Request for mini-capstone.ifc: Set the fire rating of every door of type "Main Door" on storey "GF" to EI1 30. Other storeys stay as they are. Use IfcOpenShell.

First a look at what the model holds.

```python
import ifcopenshell
import ifcopenshell.util.element

model = ifcopenshell.open("mini-capstone.ifc")
print(model.schema)
storey = next(s for s in model.by_type("IfcBuildingStorey") if s.Name == "GF")
doors = [e for e in ifcopenshell.util.element.get_decomposition(storey) if e.is_a("IfcDoor")]
seen = {}
for e in doors:
    element_type = ifcopenshell.util.element.get_type(e)
    key = (element_type.Name if element_type != e and element_type else None, ifcopenshell.util.element.get_pset(e, "Pset_DoorCommon", "FireRating"))
    seen[key] = seen.get(key, 0) + 1
for (name, value), count in sorted(seen.items(), key=str):
    print(count, "x", name, "|", value)
```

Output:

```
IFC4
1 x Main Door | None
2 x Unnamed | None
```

```python
import ifcopenshell
import ifcopenshell.api.pset
import ifcopenshell.util.element

model = ifcopenshell.open("mini-capstone.ifc")

storey = next(s for s in model.by_type("IfcBuildingStorey") if s.Name == "GF")
doors = [e for e in ifcopenshell.util.element.get_decomposition(storey) if e.is_a("IfcDoor")]

count = 0
for e in doors:
    element_type = ifcopenshell.util.element.get_type(e)
    if element_type in (None, e) or element_type.Name != "Main Door":
        continue
    # add_pset returns the element's existing set when there is one.
    pset = ifcopenshell.api.pset.add_pset(model, product=e, name="Pset_DoorCommon")
    ifcopenshell.api.pset.edit_pset(model, pset=pset, properties={"FireRating": "EI1 30"})
    count += 1

print(count, "doors updated")

model.write("mini-capstone_edited.ifc")
```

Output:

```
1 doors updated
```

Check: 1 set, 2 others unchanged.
